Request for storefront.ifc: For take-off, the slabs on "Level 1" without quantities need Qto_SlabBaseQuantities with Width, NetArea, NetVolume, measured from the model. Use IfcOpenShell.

First a look at what the model holds.

```python
import ifcopenshell
import ifcopenshell.util.element
import ifcopenshell.util.unit

model = ifcopenshell.open("storefront.ifc")
print(model.schema)
for unit_type in ("LENGTHUNIT", "AREAUNIT", "VOLUMEUNIT"):
    print(unit_type, ifcopenshell.util.unit.calculate_unit_scale(model, unit_type))
storey = next(s for s in model.by_type("IfcBuildingStorey") if s.Name == "Level 1")
slabs = [e for e in ifcopenshell.util.element.get_decomposition(storey) if e.is_a("IfcSlab")]
for e in sorted(slabs, key=lambda e: e.id()):
    print(e.id(), e.is_a(), e.Name, list(ifcopenshell.util.element.get_psets(e, qtos_only=True)), sep=" | ")
```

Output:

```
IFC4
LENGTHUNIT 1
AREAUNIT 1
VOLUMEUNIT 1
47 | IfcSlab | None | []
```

```python
import ifcopenshell
import ifcopenshell.api.pset
import ifcopenshell.geom
import ifcopenshell.util.element
import ifcopenshell.util.shape
import ifcopenshell.util.unit

model = ifcopenshell.open("storefront.ifc")
unit_scale = ifcopenshell.util.unit.calculate_unit_scale(model)
area_scale = ifcopenshell.util.unit.calculate_unit_scale(model, "AREAUNIT")
volume_scale = ifcopenshell.util.unit.calculate_unit_scale(model, "VOLUMEUNIT")
settings = ifcopenshell.geom.settings()

storey = next(s for s in model.by_type("IfcBuildingStorey") if s.Name == "Level 1")
slabs = [e for e in ifcopenshell.util.element.get_decomposition(storey) if e.is_a("IfcSlab")]

for e in sorted(slabs, key=lambda e: e.id()):
    if ifcopenshell.util.element.get_psets(e, qtos_only=True, should_inherit=False):
        continue
    # Geometry comes back in metres, in the element's own axes.
    shape = ifcopenshell.geom.create_shape(settings, e)
    values = {
        "Width": ifcopenshell.util.shape.get_z(shape.geometry) / unit_scale,
        "NetArea": ifcopenshell.util.shape.get_footprint_area(shape.geometry) / area_scale,
        "NetVolume": ifcopenshell.util.shape.get_volume(shape.geometry) / volume_scale,
    }
    qto = ifcopenshell.api.pset.add_qto(model, product=e, name="Qto_SlabBaseQuantities")
    ifcopenshell.api.pset.edit_qto(model, qto=qto, properties=values)
    print(e.id(), {k: round(v, 3) for k, v in values.items()})

model.write("storefront-out.ifc")
```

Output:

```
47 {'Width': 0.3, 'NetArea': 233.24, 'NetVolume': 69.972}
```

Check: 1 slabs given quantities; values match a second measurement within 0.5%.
